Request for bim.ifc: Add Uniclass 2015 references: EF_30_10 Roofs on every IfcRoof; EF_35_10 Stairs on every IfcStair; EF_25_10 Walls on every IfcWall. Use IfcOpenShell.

First a look at what the model holds.

```python
import ifcopenshell

model = ifcopenshell.open("bim.ifc")
print(model.schema)
print("classifications:", [c.Name for c in model.by_type("IfcClassification")])
for ifc_class in ("IfcDoor", "IfcRoof", "IfcStair", "IfcWall", "IfcWindow"):
    print(ifc_class, len(model.by_type(ifc_class)))
```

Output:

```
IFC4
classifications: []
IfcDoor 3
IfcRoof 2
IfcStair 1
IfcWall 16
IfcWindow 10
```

```python
import ifcopenshell
import ifcopenshell.api.classification

model = ifcopenshell.open("bim.ifc")

system = ifcopenshell.api.classification.add_classification(model, classification="Uniclass 2015")

codes = {
    "IfcRoof": ("EF_30_10", "Roofs"),
    "IfcStair": ("EF_35_10", "Stairs"),
    "IfcWall": ("EF_25_10", "Walls"),
}
for ifc_class, (code, name) in codes.items():
    products = model.by_type(ifc_class)
    ifcopenshell.api.classification.add_reference(
        model, products=products, classification=system, identification=code, name=name
    )
    print(code, len(products))

model.write("bim_edited.ifc")
```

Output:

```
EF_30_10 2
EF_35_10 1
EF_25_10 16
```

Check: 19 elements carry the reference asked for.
